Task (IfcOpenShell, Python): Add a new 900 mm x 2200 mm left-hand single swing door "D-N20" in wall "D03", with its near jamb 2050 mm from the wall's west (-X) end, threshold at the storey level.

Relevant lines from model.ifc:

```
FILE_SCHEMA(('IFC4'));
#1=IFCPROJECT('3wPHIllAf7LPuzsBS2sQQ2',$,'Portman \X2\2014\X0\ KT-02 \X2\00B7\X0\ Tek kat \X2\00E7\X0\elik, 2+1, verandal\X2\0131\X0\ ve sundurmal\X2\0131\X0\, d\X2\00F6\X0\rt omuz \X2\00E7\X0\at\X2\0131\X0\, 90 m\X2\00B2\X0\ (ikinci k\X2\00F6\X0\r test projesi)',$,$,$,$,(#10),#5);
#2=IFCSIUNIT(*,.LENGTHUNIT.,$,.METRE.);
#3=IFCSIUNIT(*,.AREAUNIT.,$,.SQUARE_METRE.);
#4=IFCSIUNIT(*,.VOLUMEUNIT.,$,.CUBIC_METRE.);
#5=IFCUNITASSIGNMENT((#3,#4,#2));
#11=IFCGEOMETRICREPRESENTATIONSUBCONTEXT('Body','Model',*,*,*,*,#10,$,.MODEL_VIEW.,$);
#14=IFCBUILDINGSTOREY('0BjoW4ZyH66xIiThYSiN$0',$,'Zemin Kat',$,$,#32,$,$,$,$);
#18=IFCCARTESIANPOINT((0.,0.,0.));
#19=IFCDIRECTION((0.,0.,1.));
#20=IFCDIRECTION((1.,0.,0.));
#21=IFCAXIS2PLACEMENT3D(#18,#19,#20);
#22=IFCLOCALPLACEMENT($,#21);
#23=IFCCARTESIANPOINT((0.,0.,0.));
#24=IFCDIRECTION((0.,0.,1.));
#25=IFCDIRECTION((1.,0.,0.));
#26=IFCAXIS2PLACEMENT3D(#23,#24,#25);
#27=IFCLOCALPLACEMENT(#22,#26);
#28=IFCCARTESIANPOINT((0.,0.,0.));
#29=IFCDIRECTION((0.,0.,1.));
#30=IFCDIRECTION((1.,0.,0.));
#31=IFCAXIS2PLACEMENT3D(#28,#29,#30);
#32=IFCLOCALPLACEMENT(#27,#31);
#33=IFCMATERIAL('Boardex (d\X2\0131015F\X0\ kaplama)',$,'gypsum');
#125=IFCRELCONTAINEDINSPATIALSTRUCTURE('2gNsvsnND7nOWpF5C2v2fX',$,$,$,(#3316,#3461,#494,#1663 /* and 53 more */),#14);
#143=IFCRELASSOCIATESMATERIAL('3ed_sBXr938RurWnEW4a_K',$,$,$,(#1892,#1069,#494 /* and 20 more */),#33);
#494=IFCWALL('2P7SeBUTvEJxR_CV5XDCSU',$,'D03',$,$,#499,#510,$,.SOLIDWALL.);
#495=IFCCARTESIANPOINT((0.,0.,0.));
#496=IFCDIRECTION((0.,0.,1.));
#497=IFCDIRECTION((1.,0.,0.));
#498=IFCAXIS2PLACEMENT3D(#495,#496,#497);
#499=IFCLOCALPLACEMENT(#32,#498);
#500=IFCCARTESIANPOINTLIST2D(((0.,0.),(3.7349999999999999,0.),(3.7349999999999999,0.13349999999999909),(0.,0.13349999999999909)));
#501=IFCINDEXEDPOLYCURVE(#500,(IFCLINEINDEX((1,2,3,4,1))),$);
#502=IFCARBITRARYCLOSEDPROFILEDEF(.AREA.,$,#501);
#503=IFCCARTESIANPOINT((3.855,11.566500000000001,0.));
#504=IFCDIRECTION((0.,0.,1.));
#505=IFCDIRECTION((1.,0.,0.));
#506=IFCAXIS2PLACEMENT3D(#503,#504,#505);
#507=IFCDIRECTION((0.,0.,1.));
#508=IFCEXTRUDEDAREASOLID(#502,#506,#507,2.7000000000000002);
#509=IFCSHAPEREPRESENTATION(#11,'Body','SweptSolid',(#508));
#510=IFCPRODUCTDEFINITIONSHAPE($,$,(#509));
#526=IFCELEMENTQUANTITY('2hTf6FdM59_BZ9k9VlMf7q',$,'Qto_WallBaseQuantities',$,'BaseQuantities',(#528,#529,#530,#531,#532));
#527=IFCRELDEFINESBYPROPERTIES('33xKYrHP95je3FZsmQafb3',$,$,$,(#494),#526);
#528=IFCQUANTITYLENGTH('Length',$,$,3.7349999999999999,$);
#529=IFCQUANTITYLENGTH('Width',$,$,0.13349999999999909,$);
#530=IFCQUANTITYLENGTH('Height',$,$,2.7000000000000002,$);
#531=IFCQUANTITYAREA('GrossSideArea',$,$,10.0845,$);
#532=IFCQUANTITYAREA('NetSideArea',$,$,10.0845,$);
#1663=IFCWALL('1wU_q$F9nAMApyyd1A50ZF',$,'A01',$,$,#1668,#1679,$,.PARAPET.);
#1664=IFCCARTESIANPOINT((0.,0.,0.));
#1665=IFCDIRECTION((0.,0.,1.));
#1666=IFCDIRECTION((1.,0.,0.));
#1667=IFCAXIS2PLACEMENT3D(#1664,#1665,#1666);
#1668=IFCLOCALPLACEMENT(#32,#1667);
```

```python
import numpy as np
import ifcopenshell
import ifcopenshell.api.feature
import ifcopenshell.api.geometry
import ifcopenshell.api.pset
import ifcopenshell.api.root
import ifcopenshell.api.spatial
import ifcopenshell.geom
import ifcopenshell.util.element
import ifcopenshell.util.placement
import ifcopenshell.util.representation
import ifcopenshell.util.shape
import ifcopenshell.util.unit

model = ifcopenshell.open("model.ifc")
unit_scale = ifcopenshell.util.unit.calculate_unit_scale(model)
area_scale = ifcopenshell.util.unit.calculate_unit_scale(model, "AREAUNIT")
settings = ifcopenshell.geom.settings()


def volume(element):
    """Net volume in cubic metres, openings subtracted."""
    shape = ifcopenshell.geom.create_shape(settings, element)
    return ifcopenshell.util.shape.get_volume(shape.geometry)


wall = model.by_guid("2P7SeBUTvEJxR_CV5XDCSU")
storey = ifcopenshell.util.element.get_container(wall, ifc_class="IfcBuildingStorey")
context = ifcopenshell.util.representation.get_context(model, "Model", "Body", "MODEL_VIEW")
before = volume(wall)

width, height, from_end, sill = 0.9, 2.2, 2.05, 0.0  # metres

# The wall runs along its own X axis, and the end named is its -X end.
wall_shape = ifcopenshell.geom.create_shape(settings, wall)
x, y, z = ifcopenshell.util.shape.get_vertices(wall_shape.geometry).T
start = x.min() + from_end
face, thickness = float(y.min()), float(y.max() - y.min())
wall_matrix = ifcopenshell.util.placement.get_local_placement(wall.ObjectPlacement)
level = ifcopenshell.util.placement.get_local_placement(storey.ObjectPlacement)[2, 3]


def in_wall(x, y):
    """Placement at x, y metres in the wall's axes, at sill height."""
    matrix = wall_matrix.copy()
    matrix[:, 3] = wall_matrix @ np.array([x / unit_scale, y / unit_scale, 0.0, 1.0])
    matrix[2, 3] = level + sill / unit_scale
    return matrix


# Opening: a box that overshoots both wall faces by 50 mm.
opening = ifcopenshell.api.root.create_entity(model, ifc_class="IfcOpeningElement", predefined_type="OPENING")
box = ifcopenshell.api.geometry.add_wall_representation(
    model, context=context, length=width, height=height, thickness=thickness + 0.1
)
ifcopenshell.api.geometry.assign_representation(model, product=opening, representation=box)
ifcopenshell.api.geometry.edit_object_placement(model, product=opening, matrix=in_wall(start, face - 0.05), is_si=False)
ifcopenshell.api.feature.add_feature(model, feature=opening, element=wall)

door = ifcopenshell.api.root.create_entity(model, ifc_class="IfcDoor", name="D-N20", predefined_type="DOOR")
door.OverallWidth, door.OverallHeight = width / unit_scale, height / unit_scale
door.OperationType = "SINGLE_SWING_LEFT"
body = ifcopenshell.api.geometry.add_door_representation(
    model,
    context=context,
    overall_width=door.OverallWidth,
    overall_height=door.OverallHeight,
    operation_type="SINGLE_SWING_LEFT",
    lining_properties={"LiningDepth": thickness / unit_scale, "ThresholdDepth": thickness / unit_scale},
)
ifcopenshell.api.geometry.assign_representation(model, product=door, representation=body)
ifcopenshell.api.spatial.assign_container(model, products=[door], relating_structure=storey)
ifcopenshell.api.feature.add_filling(model, opening=opening, element=door)

# The lining spans the wall, so the door starts at the wall face.
ifcopenshell.api.geometry.edit_object_placement(model, product=door, matrix=in_wall(start, face), is_si=False)

after = volume(wall)

# Update the wall's stored quantities.
qto = model.by_id(ifcopenshell.util.element.get_pset(wall, "Qto_WallBaseQuantities", should_inherit=False)["id"])
ifcopenshell.api.pset.edit_qto(model, qto=qto, properties={"NetSideArea": after / thickness / area_scale})

print(f"wall volume {before:.3f} -> {after:.3f} m3")

model.write("model_updated.ifc")
```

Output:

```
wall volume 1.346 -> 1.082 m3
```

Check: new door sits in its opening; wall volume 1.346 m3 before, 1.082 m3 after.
